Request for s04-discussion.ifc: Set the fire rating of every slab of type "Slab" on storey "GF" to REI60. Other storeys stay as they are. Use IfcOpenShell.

First a look at what the model holds.

```python
import ifcopenshell
import ifcopenshell.util.element

model = ifcopenshell.open("s04-discussion.ifc")
print(model.schema)
storey = next(s for s in model.by_type("IfcBuildingStorey") if s.Name == "GF")
slabs = [e for e in ifcopenshell.util.element.get_decomposition(storey) if e.is_a("IfcSlab")]
seen = {}
for e in slabs:
    element_type = ifcopenshell.util.element.get_type(e)
    key = (element_type.Name if element_type != e and element_type else None, ifcopenshell.util.element.get_pset(e, "Pset_SlabCommon", "FireRating"))
    seen[key] = seen.get(key, 0) + 1
for (name, value), count in sorted(seen.items(), key=str):
    print(count, "x", name, "|", value)
```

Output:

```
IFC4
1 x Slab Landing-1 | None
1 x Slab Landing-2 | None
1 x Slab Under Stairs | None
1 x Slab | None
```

```python
import ifcopenshell
import ifcopenshell.api.pset
import ifcopenshell.util.element

model = ifcopenshell.open("s04-discussion.ifc")

storey = next(s for s in model.by_type("IfcBuildingStorey") if s.Name == "GF")
slabs = [e for e in ifcopenshell.util.element.get_decomposition(storey) if e.is_a("IfcSlab")]

count = 0
for e in slabs:
    element_type = ifcopenshell.util.element.get_type(e)
    if element_type in (None, e) or element_type.Name != "Slab":
        continue
    # add_pset returns the element's existing set when there is one.
    pset = ifcopenshell.api.pset.add_pset(model, product=e, name="Pset_SlabCommon")
    ifcopenshell.api.pset.edit_pset(model, pset=pset, properties={"FireRating": "REI60"})
    count += 1

print(count, "slabs updated")

model.write("s04-discussion_edited.ifc")
```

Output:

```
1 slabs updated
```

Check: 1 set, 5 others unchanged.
